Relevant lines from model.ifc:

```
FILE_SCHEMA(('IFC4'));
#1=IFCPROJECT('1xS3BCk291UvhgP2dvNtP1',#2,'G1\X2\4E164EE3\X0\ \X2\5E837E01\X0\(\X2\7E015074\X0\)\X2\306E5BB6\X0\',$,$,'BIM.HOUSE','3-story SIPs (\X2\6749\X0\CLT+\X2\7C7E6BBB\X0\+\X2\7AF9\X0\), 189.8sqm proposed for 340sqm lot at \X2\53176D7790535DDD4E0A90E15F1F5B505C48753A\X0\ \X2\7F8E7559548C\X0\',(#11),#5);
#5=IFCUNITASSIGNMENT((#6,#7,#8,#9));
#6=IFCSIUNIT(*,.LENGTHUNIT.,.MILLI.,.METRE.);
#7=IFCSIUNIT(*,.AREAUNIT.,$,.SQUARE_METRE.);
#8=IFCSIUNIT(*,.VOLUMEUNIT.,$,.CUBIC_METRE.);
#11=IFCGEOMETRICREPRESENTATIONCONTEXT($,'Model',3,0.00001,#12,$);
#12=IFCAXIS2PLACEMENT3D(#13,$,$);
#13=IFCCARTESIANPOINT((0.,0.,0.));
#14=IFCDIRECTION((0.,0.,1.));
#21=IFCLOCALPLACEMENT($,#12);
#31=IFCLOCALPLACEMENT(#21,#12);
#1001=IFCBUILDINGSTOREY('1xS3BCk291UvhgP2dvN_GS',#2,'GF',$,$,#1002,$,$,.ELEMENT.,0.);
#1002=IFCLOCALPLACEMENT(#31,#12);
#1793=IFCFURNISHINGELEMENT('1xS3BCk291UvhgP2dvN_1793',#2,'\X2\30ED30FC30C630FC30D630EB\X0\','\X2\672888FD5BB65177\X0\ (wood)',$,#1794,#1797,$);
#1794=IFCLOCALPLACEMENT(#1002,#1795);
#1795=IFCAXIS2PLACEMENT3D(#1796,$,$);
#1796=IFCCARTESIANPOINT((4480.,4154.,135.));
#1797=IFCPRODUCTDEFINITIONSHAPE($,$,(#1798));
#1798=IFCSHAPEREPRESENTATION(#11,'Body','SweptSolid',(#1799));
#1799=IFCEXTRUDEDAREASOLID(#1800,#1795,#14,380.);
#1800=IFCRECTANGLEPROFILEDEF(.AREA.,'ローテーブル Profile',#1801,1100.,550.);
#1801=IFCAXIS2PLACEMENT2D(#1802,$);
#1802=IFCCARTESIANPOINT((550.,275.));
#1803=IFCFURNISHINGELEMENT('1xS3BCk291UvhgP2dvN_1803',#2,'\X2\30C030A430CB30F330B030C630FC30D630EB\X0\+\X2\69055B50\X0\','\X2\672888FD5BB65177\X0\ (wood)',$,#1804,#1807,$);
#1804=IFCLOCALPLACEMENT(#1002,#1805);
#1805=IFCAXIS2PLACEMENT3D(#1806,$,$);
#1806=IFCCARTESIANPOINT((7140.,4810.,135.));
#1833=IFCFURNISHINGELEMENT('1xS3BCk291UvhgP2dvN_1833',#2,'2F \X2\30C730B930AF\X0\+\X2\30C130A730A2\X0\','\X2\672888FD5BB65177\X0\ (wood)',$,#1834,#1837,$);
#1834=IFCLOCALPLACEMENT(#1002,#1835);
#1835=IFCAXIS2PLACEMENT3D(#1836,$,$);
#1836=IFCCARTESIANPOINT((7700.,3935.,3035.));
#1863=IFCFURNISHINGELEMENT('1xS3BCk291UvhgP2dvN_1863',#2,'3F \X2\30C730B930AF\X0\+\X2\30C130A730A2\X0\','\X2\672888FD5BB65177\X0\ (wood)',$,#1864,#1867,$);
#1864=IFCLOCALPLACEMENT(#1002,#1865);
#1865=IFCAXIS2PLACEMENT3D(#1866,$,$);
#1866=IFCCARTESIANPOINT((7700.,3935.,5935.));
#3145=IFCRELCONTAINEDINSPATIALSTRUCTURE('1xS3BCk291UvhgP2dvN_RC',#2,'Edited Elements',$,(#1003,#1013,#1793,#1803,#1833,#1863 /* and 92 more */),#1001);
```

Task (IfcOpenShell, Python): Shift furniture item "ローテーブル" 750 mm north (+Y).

```python
import ifcopenshell
import ifcopenshell.api.geometry
import ifcopenshell.util.placement
import ifcopenshell.util.unit

model = ifcopenshell.open("model.ifc")
unit_scale = ifcopenshell.util.unit.calculate_unit_scale(model)

item = model.by_id(1793)
matrix = ifcopenshell.util.placement.get_local_placement(item.ObjectPlacement)
matrix[1, 3] += 0.75 / unit_scale
ifcopenshell.api.geometry.edit_object_placement(model, product=item, matrix=matrix, is_si=False)

print(ifcopenshell.util.placement.get_local_placement(item.ObjectPlacement).round(3) + 0.0)

model.write("model_v2.ifc")
```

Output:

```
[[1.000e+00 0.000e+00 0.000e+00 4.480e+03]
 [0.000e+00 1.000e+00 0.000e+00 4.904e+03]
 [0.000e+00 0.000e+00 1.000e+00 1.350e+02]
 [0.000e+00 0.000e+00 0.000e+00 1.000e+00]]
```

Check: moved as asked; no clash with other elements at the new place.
